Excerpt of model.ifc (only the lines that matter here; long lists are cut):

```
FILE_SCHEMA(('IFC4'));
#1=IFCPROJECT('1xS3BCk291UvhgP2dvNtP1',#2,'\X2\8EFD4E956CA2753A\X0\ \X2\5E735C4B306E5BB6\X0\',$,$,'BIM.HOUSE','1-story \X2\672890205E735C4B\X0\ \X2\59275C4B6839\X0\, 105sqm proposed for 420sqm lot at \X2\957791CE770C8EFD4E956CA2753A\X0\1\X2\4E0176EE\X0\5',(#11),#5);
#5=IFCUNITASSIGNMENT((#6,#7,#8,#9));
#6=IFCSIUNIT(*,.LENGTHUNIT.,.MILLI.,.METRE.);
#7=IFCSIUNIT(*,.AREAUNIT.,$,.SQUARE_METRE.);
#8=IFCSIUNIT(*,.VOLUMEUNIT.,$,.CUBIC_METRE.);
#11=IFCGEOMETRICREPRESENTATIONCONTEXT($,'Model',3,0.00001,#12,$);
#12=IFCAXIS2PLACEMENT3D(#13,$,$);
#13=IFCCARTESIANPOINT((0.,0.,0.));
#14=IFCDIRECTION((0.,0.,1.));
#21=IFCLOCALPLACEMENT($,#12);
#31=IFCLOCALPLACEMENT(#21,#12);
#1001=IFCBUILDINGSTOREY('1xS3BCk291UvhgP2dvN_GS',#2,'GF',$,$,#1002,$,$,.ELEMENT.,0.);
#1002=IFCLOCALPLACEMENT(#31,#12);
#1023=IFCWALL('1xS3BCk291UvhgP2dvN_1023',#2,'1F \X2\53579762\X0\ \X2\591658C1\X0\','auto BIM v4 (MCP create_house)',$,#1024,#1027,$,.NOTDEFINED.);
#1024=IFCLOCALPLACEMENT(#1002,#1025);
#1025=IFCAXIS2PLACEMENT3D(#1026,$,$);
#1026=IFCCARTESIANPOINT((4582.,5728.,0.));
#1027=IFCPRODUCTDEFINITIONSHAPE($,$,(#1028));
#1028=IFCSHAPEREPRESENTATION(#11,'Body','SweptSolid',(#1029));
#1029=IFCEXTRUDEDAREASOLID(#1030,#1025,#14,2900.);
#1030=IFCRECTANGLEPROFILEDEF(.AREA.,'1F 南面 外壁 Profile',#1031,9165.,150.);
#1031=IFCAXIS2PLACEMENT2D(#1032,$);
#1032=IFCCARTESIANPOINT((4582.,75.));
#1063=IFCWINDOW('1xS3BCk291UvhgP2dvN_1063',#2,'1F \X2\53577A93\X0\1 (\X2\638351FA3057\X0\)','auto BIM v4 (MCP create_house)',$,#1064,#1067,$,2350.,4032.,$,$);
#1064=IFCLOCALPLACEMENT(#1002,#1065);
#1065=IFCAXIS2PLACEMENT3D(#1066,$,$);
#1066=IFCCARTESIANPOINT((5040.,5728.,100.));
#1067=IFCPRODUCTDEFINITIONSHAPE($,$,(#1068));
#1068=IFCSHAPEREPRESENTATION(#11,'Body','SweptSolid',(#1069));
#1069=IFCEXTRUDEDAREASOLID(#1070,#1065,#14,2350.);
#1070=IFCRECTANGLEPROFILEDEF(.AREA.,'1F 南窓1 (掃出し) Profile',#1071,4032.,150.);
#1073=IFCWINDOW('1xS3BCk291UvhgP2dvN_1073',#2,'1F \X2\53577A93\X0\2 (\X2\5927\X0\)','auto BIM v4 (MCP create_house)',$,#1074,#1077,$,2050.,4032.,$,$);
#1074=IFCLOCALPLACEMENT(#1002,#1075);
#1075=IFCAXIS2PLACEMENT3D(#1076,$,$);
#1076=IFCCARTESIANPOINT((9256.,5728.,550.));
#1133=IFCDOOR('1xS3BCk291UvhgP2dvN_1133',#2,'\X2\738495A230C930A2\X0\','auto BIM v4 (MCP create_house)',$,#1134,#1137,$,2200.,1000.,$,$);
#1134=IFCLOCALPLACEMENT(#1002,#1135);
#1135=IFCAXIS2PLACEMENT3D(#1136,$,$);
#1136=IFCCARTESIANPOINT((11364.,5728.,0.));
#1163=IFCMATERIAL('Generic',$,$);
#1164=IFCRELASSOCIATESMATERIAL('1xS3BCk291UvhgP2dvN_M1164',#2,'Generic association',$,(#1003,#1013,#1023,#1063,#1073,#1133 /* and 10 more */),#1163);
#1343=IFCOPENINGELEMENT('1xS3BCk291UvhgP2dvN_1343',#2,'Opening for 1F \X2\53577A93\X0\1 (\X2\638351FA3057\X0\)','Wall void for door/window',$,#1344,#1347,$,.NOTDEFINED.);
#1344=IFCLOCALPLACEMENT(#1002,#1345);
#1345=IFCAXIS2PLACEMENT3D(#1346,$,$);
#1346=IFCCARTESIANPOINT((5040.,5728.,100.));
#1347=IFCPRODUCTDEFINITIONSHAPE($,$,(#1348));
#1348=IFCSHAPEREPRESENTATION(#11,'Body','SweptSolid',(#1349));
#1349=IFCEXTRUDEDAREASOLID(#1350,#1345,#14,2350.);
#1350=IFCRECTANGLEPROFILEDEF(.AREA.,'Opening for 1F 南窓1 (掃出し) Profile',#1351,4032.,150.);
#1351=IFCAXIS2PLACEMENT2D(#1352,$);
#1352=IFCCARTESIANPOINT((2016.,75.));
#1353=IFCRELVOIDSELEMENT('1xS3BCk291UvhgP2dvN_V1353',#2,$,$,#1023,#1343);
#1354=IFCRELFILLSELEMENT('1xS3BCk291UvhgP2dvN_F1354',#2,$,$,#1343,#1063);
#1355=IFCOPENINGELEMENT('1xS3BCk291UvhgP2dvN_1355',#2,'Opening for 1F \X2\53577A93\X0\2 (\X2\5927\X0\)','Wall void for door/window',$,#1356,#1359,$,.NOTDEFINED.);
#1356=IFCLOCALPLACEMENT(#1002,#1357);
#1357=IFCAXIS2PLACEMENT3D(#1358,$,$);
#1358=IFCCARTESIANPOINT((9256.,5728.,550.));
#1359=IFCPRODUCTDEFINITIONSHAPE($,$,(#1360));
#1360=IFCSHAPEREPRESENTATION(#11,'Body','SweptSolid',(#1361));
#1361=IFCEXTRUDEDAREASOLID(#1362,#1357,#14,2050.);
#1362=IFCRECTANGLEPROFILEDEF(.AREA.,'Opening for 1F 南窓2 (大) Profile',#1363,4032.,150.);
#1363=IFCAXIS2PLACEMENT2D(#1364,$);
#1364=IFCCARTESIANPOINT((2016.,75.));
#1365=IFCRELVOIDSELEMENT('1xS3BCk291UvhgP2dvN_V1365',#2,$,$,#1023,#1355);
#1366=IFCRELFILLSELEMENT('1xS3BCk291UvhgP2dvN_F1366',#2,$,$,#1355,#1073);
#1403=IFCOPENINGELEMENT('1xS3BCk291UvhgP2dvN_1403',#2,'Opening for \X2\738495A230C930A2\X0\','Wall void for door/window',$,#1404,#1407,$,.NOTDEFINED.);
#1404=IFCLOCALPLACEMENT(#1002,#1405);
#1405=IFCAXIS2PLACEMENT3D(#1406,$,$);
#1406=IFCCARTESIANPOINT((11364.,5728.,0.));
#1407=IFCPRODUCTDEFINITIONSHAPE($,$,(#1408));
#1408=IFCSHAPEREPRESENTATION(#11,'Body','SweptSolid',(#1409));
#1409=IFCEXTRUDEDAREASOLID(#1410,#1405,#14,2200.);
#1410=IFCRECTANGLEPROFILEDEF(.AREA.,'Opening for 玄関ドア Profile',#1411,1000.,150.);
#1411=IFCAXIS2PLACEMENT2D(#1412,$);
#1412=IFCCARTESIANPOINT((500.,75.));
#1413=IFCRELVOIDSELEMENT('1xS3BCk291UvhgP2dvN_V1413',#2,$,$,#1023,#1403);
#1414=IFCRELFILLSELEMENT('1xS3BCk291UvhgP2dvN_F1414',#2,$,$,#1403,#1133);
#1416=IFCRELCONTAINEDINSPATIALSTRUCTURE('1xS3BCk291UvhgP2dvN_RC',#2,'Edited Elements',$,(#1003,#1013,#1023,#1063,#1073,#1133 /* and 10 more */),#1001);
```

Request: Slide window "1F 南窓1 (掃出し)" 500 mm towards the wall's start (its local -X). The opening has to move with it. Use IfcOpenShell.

```python
import ifcopenshell
import ifcopenshell.api.geometry
import ifcopenshell.util.placement
import ifcopenshell.util.unit

model = ifcopenshell.open("model.ifc")
unit_scale = ifcopenshell.util.unit.calculate_unit_scale(model)

window = model.by_id(1063)
opening = window.FillsVoids[0].RelatingOpeningElement
wall = opening.VoidsElements[0].RelatingBuildingElement

wall_matrix = ifcopenshell.util.placement.get_local_placement(wall.ObjectPlacement)
shift = wall_matrix[:3, 0] * -0.5 / unit_scale
before = ifcopenshell.util.placement.get_local_placement(window.ObjectPlacement)[:3, 3].copy()

# The window is not placed relative to its opening, so move both.
for product in (opening, window):
    matrix = ifcopenshell.util.placement.get_local_placement(product.ObjectPlacement)
    matrix[:3, 3] += shift
    ifcopenshell.api.geometry.edit_object_placement(model, product=product, matrix=matrix, is_si=False)

after = ifcopenshell.util.placement.get_local_placement(window.ObjectPlacement)[:3, 3]
print("window moved by", (after - before).round(3) + 0.0)

model.write("model_edited.ifc")
```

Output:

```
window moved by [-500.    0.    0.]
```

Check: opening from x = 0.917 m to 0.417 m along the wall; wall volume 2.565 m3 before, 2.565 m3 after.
